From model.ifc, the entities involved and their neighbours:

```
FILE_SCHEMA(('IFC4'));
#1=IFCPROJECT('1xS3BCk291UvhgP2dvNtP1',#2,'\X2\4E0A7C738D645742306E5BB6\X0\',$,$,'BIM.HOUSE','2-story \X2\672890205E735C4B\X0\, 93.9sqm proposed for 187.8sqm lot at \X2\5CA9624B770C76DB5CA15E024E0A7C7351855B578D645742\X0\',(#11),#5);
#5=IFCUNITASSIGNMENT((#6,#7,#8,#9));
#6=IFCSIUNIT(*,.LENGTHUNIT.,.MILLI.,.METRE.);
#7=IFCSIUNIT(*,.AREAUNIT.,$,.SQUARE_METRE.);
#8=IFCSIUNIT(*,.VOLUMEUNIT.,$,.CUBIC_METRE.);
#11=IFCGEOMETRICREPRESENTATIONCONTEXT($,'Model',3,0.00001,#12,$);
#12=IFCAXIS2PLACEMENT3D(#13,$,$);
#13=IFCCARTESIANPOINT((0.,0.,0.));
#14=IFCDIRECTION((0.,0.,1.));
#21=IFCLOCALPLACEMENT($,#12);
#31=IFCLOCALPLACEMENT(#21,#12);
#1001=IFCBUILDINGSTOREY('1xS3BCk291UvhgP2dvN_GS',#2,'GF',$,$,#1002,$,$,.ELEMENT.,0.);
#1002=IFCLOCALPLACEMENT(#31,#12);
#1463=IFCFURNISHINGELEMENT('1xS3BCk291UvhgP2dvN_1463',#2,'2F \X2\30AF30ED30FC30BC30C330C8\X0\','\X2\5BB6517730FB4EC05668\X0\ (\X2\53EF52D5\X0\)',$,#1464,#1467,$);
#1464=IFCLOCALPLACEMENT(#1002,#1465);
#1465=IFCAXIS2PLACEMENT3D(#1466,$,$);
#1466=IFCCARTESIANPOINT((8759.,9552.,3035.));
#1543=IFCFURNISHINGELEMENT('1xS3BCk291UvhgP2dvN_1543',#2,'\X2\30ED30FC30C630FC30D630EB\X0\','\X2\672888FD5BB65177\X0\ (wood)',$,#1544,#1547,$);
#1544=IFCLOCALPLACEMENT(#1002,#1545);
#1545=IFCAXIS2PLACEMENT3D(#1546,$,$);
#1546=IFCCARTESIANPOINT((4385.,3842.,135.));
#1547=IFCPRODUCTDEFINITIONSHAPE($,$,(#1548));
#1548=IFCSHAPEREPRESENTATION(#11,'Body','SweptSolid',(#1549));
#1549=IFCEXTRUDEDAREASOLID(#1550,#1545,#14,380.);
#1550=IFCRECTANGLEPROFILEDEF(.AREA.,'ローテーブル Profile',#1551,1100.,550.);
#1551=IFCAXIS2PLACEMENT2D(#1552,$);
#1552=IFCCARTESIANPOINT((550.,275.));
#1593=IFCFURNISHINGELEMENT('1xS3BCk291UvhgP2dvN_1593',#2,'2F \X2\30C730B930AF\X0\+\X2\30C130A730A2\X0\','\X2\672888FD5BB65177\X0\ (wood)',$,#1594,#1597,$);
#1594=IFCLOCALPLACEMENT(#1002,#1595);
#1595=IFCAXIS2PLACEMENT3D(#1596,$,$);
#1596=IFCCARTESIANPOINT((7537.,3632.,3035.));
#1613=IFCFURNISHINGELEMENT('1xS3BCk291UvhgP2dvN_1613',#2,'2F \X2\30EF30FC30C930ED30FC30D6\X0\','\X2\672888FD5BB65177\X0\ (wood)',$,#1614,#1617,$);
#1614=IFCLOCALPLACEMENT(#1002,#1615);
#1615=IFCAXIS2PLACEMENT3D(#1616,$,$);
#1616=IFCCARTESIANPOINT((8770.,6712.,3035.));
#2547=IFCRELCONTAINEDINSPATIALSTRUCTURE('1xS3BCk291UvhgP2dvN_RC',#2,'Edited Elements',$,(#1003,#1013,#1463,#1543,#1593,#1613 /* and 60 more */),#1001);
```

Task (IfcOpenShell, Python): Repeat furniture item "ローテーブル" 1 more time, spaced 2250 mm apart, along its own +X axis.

```python
import ifcopenshell
import ifcopenshell.api.geometry
import ifcopenshell.api.root
import ifcopenshell.util.element
import ifcopenshell.util.placement
import ifcopenshell.util.unit

model = ifcopenshell.open("model.ifc")
unit_scale = ifcopenshell.util.unit.calculate_unit_scale(model)


def reuse_history(source, copy):
    """copy_class also copies each property set's owner history, people and application; keep the originals."""
    for rel in copy.IsDefinedBy:
        if rel.is_a("IfcRelDefinesByProperties") and (history := rel.RelatingPropertyDefinition.OwnerHistory):
            rel.RelatingPropertyDefinition.OwnerHistory = source.OwnerHistory
            ifcopenshell.util.element.remove_deep2(model, history)


source = model.by_guid("1xS3BCk291UvhgP2dvN_1543")
base = ifcopenshell.util.placement.get_local_placement(source.ObjectPlacement)
step = base[:3, 0] * 2.25 / unit_scale

for i in range(1, 2):
    copy = ifcopenshell.api.root.copy_class(model, product=source)
    copy.Representation = ifcopenshell.util.element.copy_deep(
        model, source.Representation, exclude=["IfcGeometricRepresentationContext", "IfcRepresentationMap"]
    )
    reuse_history(source, copy)
    matrix = base.copy()
    matrix[:3, 3] += i * step
    print("added at", matrix[:3, 3].round(3) + 0.0)
    ifcopenshell.api.geometry.edit_object_placement(model, product=copy, matrix=matrix, is_si=False)

model.write("model-out.ifc")
```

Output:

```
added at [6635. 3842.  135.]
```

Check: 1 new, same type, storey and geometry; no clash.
